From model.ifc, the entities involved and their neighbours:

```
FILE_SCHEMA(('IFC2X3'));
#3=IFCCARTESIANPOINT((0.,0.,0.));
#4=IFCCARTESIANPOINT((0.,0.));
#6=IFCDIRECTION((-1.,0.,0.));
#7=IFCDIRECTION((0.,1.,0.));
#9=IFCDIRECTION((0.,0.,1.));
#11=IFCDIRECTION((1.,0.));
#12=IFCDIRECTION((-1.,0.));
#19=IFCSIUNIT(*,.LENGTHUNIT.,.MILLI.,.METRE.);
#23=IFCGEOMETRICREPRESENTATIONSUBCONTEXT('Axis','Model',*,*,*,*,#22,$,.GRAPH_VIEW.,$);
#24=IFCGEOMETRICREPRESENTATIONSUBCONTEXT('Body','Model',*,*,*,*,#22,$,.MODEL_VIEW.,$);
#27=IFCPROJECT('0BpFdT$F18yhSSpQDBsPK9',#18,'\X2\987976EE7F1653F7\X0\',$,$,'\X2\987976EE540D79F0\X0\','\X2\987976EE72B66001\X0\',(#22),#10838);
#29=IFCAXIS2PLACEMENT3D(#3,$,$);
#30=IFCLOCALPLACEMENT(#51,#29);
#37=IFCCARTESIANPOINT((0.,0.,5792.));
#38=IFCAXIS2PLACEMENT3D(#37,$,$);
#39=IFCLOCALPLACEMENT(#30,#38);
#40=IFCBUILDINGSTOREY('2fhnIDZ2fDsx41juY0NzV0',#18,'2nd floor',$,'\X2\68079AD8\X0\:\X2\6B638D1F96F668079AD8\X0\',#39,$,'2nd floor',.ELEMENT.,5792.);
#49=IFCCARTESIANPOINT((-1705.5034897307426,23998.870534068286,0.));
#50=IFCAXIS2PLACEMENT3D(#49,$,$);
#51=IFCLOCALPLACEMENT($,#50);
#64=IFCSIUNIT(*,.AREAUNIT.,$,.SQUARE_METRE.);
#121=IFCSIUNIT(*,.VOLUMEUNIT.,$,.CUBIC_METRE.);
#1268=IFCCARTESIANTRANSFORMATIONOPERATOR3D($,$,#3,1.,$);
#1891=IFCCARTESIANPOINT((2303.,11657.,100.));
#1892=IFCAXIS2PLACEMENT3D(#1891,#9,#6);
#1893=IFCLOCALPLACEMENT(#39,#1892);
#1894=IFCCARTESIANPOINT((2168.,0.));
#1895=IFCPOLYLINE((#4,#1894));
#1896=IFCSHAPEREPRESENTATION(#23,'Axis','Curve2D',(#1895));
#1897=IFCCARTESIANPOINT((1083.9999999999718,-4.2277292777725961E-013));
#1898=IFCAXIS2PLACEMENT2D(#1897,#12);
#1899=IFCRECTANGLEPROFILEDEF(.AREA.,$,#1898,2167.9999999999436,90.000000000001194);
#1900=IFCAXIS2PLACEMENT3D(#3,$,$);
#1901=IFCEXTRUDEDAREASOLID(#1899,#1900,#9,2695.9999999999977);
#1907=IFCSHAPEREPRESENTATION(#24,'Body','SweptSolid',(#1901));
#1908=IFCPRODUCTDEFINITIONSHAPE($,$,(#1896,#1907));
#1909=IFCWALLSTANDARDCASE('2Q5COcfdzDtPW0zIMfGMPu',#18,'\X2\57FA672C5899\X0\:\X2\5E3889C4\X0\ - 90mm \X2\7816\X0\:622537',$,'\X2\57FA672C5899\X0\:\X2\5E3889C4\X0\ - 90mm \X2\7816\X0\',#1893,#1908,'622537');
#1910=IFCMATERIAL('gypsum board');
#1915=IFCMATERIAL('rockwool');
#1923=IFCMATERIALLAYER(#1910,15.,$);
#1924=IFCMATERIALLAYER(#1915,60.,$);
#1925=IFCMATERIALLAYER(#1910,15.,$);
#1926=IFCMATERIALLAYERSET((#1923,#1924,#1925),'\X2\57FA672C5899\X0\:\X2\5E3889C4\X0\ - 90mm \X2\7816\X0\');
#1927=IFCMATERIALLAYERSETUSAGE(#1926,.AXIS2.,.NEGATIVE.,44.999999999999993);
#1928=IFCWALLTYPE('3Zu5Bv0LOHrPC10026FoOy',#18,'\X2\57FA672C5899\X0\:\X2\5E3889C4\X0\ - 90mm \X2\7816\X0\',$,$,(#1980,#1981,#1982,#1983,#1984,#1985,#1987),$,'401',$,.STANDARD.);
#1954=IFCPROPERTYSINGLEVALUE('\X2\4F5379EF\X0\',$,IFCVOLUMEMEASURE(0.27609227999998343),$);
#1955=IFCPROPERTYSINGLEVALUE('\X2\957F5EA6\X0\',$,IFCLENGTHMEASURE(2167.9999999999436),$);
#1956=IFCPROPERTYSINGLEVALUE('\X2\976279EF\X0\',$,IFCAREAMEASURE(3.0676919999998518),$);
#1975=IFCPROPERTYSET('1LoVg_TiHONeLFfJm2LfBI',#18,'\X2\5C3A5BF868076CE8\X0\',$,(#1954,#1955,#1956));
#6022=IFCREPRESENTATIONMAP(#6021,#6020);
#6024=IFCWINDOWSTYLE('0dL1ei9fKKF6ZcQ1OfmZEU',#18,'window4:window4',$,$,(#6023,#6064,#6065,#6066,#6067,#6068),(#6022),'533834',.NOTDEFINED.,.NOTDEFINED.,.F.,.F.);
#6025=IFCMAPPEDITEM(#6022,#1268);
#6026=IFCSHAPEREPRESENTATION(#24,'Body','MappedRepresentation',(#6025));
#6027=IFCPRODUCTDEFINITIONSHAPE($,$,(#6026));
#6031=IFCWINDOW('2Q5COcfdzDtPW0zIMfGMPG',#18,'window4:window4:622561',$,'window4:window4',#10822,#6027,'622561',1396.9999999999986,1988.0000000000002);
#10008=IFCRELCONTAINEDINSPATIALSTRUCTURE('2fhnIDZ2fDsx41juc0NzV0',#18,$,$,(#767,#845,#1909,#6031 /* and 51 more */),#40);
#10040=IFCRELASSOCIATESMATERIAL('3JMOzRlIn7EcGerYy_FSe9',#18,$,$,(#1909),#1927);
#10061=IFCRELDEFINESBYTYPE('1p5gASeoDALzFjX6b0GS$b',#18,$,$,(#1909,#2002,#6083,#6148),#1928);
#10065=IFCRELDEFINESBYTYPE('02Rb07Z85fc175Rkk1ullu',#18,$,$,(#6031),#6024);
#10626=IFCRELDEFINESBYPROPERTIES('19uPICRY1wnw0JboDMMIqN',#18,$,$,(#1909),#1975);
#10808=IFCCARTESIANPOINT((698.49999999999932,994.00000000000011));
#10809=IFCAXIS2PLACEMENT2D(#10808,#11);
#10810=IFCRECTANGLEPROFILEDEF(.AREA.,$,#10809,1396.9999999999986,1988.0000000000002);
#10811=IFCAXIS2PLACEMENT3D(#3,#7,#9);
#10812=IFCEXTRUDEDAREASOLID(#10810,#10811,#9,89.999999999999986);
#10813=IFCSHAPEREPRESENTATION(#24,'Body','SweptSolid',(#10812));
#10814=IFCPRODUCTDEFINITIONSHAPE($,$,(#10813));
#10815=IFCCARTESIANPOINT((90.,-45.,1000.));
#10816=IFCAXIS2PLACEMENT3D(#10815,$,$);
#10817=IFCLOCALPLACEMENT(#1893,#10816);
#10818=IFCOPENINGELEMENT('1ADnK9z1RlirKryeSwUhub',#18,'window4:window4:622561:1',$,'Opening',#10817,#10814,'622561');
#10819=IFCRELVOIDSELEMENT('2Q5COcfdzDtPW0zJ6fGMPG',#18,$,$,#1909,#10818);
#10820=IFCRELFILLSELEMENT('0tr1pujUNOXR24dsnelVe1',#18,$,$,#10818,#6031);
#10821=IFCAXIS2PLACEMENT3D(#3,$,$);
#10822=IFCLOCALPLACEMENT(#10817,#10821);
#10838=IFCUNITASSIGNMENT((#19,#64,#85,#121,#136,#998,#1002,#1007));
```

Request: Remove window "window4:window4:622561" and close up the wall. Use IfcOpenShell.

```python
import ifcopenshell
import ifcopenshell.api.feature
import ifcopenshell.api.pset
import ifcopenshell.api.root
import ifcopenshell.geom
import ifcopenshell.util.element
import ifcopenshell.util.shape
import ifcopenshell.util.unit

model = ifcopenshell.open("model.ifc")
area_scale = ifcopenshell.util.unit.calculate_unit_scale(model, "AREAUNIT")
volume_scale = ifcopenshell.util.unit.calculate_unit_scale(model, "VOLUMEUNIT")
settings = ifcopenshell.geom.settings()


def volume(element):
    """Net volume in cubic metres, openings subtracted."""
    shape = ifcopenshell.geom.create_shape(settings, element)
    return ifcopenshell.util.shape.get_volume(shape.geometry)


window = model.by_guid("2Q5COcfdzDtPW0zIMfGMPG")
opening = window.FillsVoids[0].RelatingOpeningElement
wall = opening.VoidsElements[0].RelatingBuildingElement
before = volume(wall)

ifcopenshell.api.root.remove_product(model, product=window)
ifcopenshell.api.feature.remove_feature(model, feature=opening)

after = volume(wall)
thickness = 0.09  # wall thickness in metres

# Update the wall's stored quantities.
pset = model.by_id(ifcopenshell.util.element.get_pset(wall, "尺寸标注", should_inherit=False)["id"])
ifcopenshell.api.pset.edit_pset(model, pset=pset, properties={
    "体积": model.create_entity("IfcVolumeMeasure", after / volume_scale),
    "面积": model.create_entity("IfcAreaMeasure", after / thickness / area_scale),
})

print(f"wall volume {before:.3f} -> {after:.3f} m3")

model.write("model_updated.ifc")
```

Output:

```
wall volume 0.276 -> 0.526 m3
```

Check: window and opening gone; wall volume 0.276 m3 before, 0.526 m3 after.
